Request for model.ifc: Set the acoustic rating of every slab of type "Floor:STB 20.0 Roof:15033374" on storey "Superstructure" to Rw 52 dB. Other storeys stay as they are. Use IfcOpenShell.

First a look at what the model holds.

```python
import ifcopenshell
import ifcopenshell.util.element

model = ifcopenshell.open("model.ifc")
print(model.schema)
storey = next(s for s in model.by_type("IfcBuildingStorey") if s.Name == "Superstructure")
slabs = [e for e in ifcopenshell.util.element.get_decomposition(storey) if e.is_a("IfcSlab")]
seen = {}
for e in slabs:
    element_type = ifcopenshell.util.element.get_type(e)
    key = (element_type.Name if element_type != e and element_type else None, ifcopenshell.util.element.get_pset(e, "Pset_SlabCommon", "AcousticRating"))
    seen[key] = seen.get(key, 0) + 1
for (name, value), count in sorted(seen.items(), key=str):
    print(count, "x", name, "|", value)
```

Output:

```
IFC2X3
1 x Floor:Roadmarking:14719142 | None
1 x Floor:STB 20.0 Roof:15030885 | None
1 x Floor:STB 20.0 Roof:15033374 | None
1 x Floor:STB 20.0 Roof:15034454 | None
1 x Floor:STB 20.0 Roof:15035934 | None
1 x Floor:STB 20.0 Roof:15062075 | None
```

```python
import ifcopenshell
import ifcopenshell.api.pset
import ifcopenshell.util.element

model = ifcopenshell.open("model.ifc")

storey = next(s for s in model.by_type("IfcBuildingStorey") if s.Name == "Superstructure")
slabs = [e for e in ifcopenshell.util.element.get_decomposition(storey) if e.is_a("IfcSlab")]

count = 0
for e in slabs:
    element_type = ifcopenshell.util.element.get_type(e)
    if element_type in (None, e) or element_type.Name != "Floor:STB 20.0 Roof:15033374":
        continue
    # add_pset returns the element's existing set when there is one.
    pset = ifcopenshell.api.pset.add_pset(model, product=e, name="Pset_SlabCommon")
    ifcopenshell.api.pset.edit_pset(model, pset=pset, properties={"AcousticRating": "Rw 52 dB"})
    count += 1

print(count, "slabs updated")

model.write("model_updated.ifc")
```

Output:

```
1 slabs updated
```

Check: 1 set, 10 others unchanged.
